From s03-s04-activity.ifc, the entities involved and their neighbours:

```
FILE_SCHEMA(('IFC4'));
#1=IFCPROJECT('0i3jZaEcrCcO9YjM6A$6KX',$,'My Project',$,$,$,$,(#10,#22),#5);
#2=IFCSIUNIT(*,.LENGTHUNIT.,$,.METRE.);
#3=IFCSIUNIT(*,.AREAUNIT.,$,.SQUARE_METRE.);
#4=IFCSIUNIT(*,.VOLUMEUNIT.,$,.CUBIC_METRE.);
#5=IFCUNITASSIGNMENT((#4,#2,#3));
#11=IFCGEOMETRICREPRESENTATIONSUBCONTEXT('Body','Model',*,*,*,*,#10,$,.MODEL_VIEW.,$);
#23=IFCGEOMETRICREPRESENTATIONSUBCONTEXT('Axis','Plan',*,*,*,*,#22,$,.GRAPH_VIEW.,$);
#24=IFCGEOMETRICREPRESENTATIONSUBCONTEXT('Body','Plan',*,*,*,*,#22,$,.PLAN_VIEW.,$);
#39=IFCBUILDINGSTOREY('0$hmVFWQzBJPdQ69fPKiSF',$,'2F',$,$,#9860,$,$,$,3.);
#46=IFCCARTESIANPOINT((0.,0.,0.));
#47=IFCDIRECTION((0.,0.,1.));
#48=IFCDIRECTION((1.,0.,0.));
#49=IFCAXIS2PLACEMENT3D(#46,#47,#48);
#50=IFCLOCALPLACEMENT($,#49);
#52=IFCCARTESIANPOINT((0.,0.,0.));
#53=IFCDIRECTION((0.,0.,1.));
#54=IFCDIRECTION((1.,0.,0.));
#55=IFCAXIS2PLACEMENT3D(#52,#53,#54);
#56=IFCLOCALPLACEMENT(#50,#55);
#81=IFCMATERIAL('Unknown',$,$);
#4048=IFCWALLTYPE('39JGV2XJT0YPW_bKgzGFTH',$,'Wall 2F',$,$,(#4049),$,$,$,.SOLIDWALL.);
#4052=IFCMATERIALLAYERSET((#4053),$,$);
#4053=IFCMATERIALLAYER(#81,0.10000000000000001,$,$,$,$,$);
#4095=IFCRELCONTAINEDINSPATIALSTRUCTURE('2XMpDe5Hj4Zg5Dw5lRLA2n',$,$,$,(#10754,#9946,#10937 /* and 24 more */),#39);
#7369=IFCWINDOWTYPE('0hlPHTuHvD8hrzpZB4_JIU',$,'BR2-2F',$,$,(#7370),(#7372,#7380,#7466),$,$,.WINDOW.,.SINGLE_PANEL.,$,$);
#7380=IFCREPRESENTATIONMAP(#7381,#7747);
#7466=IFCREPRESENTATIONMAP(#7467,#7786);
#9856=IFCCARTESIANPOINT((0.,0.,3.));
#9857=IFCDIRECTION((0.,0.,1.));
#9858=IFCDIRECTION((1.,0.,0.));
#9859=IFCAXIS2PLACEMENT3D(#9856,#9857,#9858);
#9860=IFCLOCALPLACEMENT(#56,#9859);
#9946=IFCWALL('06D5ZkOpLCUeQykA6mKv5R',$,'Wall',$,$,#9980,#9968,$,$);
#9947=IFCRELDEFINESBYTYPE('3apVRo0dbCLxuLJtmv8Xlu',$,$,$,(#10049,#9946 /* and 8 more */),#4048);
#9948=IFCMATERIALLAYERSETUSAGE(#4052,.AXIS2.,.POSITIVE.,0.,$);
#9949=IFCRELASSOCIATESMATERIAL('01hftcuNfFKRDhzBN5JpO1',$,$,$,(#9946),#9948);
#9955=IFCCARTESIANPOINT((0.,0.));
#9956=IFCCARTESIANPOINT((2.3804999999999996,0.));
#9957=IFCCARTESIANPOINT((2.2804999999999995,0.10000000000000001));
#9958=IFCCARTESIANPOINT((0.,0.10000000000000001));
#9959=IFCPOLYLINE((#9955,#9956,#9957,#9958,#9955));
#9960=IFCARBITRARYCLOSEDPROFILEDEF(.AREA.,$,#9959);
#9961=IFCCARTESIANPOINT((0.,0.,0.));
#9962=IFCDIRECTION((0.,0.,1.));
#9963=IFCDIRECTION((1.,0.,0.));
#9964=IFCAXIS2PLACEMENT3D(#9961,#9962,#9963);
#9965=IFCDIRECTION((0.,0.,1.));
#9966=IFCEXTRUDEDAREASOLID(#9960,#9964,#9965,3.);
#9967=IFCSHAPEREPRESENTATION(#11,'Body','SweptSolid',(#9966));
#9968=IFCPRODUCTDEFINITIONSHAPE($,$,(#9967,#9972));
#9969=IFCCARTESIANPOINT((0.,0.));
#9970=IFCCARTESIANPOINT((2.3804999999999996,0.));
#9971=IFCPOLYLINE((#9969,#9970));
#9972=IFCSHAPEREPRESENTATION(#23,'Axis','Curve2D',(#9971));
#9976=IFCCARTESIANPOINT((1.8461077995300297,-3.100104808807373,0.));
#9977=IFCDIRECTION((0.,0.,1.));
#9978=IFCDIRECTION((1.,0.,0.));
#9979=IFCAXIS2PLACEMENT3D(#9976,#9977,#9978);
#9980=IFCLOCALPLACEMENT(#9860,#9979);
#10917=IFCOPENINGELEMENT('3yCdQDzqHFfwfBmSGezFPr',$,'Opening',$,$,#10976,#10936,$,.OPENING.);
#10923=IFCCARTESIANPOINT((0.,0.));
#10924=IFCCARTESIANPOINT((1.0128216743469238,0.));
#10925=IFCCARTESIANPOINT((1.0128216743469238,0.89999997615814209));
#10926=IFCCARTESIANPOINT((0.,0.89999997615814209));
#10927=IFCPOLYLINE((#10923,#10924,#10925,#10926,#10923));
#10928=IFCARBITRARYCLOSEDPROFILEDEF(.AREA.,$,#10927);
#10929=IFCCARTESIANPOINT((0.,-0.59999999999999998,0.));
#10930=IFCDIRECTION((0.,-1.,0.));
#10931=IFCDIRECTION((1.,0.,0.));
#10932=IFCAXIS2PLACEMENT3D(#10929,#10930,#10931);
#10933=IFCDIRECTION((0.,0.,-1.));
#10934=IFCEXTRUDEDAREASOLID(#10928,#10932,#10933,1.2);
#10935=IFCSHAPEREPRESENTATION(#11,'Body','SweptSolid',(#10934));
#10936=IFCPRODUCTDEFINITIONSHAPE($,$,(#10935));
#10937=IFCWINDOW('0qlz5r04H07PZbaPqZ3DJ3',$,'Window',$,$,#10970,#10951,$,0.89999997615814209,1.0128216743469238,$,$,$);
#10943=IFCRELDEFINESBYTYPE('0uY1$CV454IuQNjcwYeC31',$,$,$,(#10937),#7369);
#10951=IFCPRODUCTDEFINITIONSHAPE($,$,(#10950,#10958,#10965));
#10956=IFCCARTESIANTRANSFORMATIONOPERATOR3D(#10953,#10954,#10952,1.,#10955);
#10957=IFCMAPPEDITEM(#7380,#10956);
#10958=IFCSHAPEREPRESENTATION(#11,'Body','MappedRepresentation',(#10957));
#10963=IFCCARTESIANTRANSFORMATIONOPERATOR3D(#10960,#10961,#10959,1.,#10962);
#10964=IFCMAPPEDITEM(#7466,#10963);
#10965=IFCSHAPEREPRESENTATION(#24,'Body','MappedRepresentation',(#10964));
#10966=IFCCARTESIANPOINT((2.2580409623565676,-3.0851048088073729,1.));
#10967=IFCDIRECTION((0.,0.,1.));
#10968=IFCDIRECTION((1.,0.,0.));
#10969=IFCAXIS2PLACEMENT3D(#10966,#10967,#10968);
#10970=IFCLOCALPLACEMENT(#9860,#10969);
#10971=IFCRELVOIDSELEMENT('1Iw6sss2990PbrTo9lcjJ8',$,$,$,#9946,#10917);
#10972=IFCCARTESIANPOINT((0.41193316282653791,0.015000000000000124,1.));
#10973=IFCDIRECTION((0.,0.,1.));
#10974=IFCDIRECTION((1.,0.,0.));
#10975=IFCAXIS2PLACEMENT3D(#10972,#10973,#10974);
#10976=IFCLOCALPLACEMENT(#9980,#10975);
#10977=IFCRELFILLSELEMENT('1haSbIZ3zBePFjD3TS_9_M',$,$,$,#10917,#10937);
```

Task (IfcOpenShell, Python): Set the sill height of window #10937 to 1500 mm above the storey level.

```python
import numpy as np
import ifcopenshell
import ifcopenshell.api.geometry
import ifcopenshell.geom
import ifcopenshell.util.element
import ifcopenshell.util.placement
import ifcopenshell.util.shape
import ifcopenshell.util.unit

model = ifcopenshell.open("s03-s04-activity.ifc")
unit_scale = ifcopenshell.util.unit.calculate_unit_scale(model)

window = model.by_id(10937)
opening = window.FillsVoids[0].RelatingOpeningElement
storey = ifcopenshell.util.element.get_container(window, ifc_class="IfcBuildingStorey")
level = ifcopenshell.util.placement.get_local_placement(storey.ObjectPlacement)[2, 3]

# The opening's origin need not be at the sill, so measure its lowest point.
shape = ifcopenshell.geom.create_shape(ifcopenshell.geom.settings(), opening)
bottom = ifcopenshell.util.shape.get_shape_bottom_elevation(shape, shape.geometry) / unit_scale
dz = level + 1.5 / unit_scale - bottom

shift = np.array([0.0, 0.0, dz])
# The window is not placed relative to its opening, so move both.
for product in (opening, window):
    matrix = ifcopenshell.util.placement.get_local_placement(product.ObjectPlacement)
    matrix[:3, 3] += shift
    ifcopenshell.api.geometry.edit_object_placement(model, product=product, matrix=matrix, is_si=False)

print(f"moved by {dz * unit_scale:+.3f} m")

model.write("s03-s04-activity_edited.ifc")
```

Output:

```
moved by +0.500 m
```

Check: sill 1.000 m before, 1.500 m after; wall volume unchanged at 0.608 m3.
